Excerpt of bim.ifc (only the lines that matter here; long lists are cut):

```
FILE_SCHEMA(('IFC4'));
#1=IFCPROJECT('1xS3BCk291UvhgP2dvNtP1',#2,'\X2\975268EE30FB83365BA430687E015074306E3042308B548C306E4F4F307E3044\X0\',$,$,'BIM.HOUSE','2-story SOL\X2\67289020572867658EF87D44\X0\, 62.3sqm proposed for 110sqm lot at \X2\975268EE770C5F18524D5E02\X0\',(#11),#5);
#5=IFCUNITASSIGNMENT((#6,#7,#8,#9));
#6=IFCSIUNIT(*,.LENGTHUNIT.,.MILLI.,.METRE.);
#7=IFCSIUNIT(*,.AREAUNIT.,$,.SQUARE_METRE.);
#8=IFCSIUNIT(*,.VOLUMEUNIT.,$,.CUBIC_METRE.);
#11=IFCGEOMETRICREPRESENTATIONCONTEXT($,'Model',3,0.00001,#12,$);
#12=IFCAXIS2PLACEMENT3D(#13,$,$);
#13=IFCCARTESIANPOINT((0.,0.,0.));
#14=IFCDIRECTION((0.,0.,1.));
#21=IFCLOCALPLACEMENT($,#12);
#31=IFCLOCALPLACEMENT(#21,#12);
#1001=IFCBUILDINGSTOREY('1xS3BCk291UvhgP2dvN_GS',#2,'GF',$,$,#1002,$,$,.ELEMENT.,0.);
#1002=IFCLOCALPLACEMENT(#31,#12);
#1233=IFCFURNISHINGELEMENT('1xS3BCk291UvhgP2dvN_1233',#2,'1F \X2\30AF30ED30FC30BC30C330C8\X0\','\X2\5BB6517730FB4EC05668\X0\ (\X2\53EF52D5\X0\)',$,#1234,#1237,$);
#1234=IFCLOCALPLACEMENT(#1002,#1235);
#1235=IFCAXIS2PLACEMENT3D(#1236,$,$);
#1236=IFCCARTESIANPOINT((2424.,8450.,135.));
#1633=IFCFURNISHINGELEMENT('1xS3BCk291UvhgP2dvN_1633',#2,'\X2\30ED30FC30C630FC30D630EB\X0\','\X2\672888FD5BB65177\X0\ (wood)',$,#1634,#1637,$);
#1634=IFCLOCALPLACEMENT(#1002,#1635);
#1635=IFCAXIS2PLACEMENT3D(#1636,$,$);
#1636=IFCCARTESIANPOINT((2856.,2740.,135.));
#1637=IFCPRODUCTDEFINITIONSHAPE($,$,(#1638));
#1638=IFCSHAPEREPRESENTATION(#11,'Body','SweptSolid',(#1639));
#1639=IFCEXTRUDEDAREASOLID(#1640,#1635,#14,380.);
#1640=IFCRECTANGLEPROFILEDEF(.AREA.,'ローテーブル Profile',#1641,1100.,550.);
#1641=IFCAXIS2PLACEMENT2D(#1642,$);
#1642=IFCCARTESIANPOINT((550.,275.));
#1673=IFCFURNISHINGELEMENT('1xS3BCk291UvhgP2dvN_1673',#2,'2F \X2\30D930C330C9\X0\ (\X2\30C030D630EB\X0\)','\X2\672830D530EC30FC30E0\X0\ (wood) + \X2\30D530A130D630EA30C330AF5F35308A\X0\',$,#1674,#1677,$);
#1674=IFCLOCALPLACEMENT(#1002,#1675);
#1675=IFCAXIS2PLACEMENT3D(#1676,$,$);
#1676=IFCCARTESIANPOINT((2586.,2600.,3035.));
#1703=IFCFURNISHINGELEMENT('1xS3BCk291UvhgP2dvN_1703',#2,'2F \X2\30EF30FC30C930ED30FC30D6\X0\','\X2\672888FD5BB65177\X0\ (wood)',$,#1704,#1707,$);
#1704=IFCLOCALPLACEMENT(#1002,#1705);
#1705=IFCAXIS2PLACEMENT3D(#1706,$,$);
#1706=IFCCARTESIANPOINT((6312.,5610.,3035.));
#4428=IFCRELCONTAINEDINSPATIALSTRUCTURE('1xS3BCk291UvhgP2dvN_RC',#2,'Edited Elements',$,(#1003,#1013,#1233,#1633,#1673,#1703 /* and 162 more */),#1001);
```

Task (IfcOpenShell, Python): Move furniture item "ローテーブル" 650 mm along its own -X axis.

```python
import ifcopenshell
import ifcopenshell.api.geometry
import ifcopenshell.util.placement
import ifcopenshell.util.unit

model = ifcopenshell.open("bim.ifc")
unit_scale = ifcopenshell.util.unit.calculate_unit_scale(model)

item = model.by_guid("1xS3BCk291UvhgP2dvN_1633")
matrix = ifcopenshell.util.placement.get_local_placement(item.ObjectPlacement)
matrix[:3, 3] -= matrix[:3, 0] * 0.65 / unit_scale
ifcopenshell.api.geometry.edit_object_placement(model, product=item, matrix=matrix, is_si=False)

print(ifcopenshell.util.placement.get_local_placement(item.ObjectPlacement).round(3) + 0.0)

model.write("bim-out.ifc")
```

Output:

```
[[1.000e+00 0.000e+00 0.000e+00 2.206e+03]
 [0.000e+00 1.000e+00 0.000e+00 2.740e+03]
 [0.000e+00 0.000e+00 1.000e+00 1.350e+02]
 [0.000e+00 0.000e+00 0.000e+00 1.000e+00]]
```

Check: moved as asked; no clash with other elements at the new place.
